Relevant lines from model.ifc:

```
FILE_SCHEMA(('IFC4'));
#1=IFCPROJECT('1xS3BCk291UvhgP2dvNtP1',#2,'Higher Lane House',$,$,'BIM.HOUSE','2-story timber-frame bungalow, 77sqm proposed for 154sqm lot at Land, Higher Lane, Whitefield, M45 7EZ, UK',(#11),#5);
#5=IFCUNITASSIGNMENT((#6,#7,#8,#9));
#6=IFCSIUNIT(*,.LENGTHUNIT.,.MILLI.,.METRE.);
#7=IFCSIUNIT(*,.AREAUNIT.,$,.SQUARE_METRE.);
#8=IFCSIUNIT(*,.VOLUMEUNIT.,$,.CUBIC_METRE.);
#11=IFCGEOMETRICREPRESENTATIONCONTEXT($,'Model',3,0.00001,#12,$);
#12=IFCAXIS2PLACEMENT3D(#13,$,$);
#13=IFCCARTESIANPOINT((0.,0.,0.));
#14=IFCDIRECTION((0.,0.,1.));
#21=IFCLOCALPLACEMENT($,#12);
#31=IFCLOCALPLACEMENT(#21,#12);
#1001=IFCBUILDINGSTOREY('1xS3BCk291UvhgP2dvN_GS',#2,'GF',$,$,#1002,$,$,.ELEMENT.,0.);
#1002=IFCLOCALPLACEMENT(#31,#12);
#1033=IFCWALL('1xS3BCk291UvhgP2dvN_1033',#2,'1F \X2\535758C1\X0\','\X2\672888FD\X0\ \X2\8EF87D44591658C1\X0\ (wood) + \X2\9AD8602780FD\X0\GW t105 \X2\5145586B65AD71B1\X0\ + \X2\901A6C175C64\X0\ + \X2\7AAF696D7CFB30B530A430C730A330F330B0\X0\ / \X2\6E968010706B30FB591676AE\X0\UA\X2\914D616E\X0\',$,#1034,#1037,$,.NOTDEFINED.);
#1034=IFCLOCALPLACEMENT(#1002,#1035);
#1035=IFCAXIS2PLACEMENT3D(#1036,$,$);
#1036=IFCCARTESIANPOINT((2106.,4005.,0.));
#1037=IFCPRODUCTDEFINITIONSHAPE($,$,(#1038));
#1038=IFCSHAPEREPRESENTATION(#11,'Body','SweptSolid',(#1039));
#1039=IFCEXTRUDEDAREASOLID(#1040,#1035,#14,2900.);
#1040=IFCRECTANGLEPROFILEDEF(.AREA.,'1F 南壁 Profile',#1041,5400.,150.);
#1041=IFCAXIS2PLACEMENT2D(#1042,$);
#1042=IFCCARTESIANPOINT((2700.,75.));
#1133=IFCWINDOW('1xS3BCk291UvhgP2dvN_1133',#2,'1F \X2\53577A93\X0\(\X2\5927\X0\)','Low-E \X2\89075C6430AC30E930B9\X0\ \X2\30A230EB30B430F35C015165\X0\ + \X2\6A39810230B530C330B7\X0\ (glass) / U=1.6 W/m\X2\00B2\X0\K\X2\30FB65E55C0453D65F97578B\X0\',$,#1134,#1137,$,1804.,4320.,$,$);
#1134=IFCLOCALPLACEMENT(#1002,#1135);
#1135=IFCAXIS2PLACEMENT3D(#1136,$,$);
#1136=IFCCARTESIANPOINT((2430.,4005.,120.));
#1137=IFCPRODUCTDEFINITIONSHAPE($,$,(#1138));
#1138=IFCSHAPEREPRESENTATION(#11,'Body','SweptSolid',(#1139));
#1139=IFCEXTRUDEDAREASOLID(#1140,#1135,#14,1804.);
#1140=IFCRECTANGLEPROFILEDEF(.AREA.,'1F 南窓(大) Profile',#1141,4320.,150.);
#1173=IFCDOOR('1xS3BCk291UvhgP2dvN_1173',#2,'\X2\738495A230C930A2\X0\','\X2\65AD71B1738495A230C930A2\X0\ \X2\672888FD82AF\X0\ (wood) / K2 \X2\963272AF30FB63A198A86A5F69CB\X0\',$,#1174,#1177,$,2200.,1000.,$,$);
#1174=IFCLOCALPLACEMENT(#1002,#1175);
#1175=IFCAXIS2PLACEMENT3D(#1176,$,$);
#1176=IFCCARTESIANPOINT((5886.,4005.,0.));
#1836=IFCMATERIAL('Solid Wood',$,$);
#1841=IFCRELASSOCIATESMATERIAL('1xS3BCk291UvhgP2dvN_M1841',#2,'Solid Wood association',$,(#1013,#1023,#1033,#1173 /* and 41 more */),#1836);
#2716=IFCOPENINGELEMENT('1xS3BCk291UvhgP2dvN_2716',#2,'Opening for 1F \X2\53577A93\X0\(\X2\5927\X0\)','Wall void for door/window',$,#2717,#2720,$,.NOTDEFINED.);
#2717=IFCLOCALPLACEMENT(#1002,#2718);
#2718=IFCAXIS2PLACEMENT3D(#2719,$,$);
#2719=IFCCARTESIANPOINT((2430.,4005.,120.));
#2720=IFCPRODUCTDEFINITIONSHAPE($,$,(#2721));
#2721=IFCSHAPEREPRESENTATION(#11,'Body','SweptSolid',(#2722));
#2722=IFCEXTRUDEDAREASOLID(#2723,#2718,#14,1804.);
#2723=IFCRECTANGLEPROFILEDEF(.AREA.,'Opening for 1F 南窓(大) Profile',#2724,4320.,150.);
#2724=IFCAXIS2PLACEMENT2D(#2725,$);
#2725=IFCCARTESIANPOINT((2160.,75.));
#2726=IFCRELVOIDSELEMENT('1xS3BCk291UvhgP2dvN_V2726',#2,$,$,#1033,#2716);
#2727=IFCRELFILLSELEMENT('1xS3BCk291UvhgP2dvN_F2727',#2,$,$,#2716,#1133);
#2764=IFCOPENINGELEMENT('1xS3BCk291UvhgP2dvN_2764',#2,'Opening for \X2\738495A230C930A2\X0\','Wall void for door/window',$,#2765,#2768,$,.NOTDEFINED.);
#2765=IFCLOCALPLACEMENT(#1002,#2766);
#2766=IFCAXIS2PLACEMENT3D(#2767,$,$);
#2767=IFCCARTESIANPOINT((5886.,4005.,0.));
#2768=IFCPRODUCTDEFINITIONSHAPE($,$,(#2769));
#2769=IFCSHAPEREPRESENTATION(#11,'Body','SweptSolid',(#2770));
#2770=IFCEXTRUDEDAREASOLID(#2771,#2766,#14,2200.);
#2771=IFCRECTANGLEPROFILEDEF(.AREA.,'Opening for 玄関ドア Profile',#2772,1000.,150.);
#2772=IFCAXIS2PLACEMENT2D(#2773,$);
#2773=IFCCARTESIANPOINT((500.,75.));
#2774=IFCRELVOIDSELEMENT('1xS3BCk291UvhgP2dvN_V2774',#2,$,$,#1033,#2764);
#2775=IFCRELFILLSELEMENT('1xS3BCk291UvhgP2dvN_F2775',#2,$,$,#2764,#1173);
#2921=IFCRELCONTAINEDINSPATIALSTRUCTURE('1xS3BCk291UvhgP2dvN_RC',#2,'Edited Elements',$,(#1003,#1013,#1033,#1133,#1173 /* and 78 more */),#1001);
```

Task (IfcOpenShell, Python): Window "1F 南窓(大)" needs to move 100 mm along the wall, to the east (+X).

```python
import ifcopenshell
import ifcopenshell.api.geometry
import ifcopenshell.util.placement

model = ifcopenshell.open("model.ifc")

window = model.by_guid("1xS3BCk291UvhgP2dvN_1133")
opening = window.FillsVoids[0].RelatingOpeningElement
wall = opening.VoidsElements[0].RelatingBuildingElement

wall_matrix = ifcopenshell.util.placement.get_local_placement(wall.ObjectPlacement)
shift = wall_matrix[:3, 0] * 100.0
before = ifcopenshell.util.placement.get_local_placement(window.ObjectPlacement)[:3, 3].copy()

# The window is not placed relative to its opening, so move both.
for product in (opening, window):
    matrix = ifcopenshell.util.placement.get_local_placement(product.ObjectPlacement)
    matrix[:3, 3] += shift
    ifcopenshell.api.geometry.edit_object_placement(model, product=product, matrix=matrix, is_si=False)

after = ifcopenshell.util.placement.get_local_placement(window.ObjectPlacement)[:3, 3]
print("window moved by", (after - before).round(3) + 0.0)

model.write("model-out.ifc")
```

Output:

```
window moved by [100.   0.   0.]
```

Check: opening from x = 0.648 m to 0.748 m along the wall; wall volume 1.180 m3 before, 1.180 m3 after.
